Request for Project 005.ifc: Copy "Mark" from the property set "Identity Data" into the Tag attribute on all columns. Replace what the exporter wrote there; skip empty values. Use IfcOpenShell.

First a look at what the model holds.

```python
import ifcopenshell
import ifcopenshell.util.element

model = ifcopenshell.open("Project 005.ifc")
print(model.schema)
columns = model.by_type("IfcColumn")
print(len(columns), "columns")
for e in columns[:8]:
    source = ifcopenshell.util.element.get_pset(e, "Identity Data", "Mark")
    target = e.Tag
    print(e.id(), repr(source), repr(target), sep=" | ")
```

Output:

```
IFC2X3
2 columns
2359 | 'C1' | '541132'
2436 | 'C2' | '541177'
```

```python
import ifcopenshell
import ifcopenshell.util.element

model = ifcopenshell.open("Project 005.ifc")

count = 0
for e in model.by_type("IfcColumn"):
    value = ifcopenshell.util.element.get_pset(e, "Identity Data", "Mark")
    current = e.Tag
    if not value or not value.strip() or current == value:
        continue
    e.Tag = value
    count += 1

print(count, "columns updated")

model.write("Project 005-out.ifc")
```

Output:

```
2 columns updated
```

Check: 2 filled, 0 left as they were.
